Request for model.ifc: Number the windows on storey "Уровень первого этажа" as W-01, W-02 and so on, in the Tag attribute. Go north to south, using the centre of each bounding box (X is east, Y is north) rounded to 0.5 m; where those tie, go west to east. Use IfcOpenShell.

First a look at what the model holds.

```python
import ifcopenshell
import ifcopenshell.util.element
import ifcopenshell.util.placement

model = ifcopenshell.open("model.ifc")
print(model.schema)
storey = next(s for s in model.by_type("IfcBuildingStorey") if s.Name == "Уровень первого этажа")
windows = [e for e in ifcopenshell.util.element.get_decomposition(storey) if e.is_a("IfcWindow")]
for e in sorted(windows, key=lambda e: e.id()):
    origin = ifcopenshell.util.placement.get_local_placement(e.ObjectPlacement)[:3, 3]
    print(e.id(), e.Tag, e.Name, origin.round(2) + 0.0, sep=" | ")
```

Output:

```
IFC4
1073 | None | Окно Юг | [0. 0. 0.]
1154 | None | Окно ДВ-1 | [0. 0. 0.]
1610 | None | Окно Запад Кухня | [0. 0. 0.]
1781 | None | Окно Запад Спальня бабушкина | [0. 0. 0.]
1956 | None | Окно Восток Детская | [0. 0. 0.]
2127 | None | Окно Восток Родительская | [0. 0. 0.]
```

```python
import ifcopenshell
import ifcopenshell.geom
import ifcopenshell.util.element
import ifcopenshell.util.shape

model = ifcopenshell.open("model.ifc")
settings = ifcopenshell.geom.settings()
settings.set("use-world-coords", True)


def centre(element):
    shape = ifcopenshell.geom.create_shape(settings, element)
    return ifcopenshell.util.shape.get_bbox_centroid(shape.geometry)


storey = next(s for s in model.by_type("IfcBuildingStorey") if s.Name == "Уровень первого этажа")
windows = [e for e in ifcopenshell.util.element.get_decomposition(storey) if e.is_a("IfcWindow")]

# Insertion points can sit at a corner or the storey origin, so sort by the geometry (in metres).
centres = {e: centre(e) for e in windows}
windows.sort(key=lambda e: (-round(centres[e][1] / 0.5), centres[e][0]))

for i, e in enumerate(windows, start=1):
    number = f"W-{i:02d}"
    e.Tag = number
    print(e.id(), number)

model.write("model_v2.ifc")
```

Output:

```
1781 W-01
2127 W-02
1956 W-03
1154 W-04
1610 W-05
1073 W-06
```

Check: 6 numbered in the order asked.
